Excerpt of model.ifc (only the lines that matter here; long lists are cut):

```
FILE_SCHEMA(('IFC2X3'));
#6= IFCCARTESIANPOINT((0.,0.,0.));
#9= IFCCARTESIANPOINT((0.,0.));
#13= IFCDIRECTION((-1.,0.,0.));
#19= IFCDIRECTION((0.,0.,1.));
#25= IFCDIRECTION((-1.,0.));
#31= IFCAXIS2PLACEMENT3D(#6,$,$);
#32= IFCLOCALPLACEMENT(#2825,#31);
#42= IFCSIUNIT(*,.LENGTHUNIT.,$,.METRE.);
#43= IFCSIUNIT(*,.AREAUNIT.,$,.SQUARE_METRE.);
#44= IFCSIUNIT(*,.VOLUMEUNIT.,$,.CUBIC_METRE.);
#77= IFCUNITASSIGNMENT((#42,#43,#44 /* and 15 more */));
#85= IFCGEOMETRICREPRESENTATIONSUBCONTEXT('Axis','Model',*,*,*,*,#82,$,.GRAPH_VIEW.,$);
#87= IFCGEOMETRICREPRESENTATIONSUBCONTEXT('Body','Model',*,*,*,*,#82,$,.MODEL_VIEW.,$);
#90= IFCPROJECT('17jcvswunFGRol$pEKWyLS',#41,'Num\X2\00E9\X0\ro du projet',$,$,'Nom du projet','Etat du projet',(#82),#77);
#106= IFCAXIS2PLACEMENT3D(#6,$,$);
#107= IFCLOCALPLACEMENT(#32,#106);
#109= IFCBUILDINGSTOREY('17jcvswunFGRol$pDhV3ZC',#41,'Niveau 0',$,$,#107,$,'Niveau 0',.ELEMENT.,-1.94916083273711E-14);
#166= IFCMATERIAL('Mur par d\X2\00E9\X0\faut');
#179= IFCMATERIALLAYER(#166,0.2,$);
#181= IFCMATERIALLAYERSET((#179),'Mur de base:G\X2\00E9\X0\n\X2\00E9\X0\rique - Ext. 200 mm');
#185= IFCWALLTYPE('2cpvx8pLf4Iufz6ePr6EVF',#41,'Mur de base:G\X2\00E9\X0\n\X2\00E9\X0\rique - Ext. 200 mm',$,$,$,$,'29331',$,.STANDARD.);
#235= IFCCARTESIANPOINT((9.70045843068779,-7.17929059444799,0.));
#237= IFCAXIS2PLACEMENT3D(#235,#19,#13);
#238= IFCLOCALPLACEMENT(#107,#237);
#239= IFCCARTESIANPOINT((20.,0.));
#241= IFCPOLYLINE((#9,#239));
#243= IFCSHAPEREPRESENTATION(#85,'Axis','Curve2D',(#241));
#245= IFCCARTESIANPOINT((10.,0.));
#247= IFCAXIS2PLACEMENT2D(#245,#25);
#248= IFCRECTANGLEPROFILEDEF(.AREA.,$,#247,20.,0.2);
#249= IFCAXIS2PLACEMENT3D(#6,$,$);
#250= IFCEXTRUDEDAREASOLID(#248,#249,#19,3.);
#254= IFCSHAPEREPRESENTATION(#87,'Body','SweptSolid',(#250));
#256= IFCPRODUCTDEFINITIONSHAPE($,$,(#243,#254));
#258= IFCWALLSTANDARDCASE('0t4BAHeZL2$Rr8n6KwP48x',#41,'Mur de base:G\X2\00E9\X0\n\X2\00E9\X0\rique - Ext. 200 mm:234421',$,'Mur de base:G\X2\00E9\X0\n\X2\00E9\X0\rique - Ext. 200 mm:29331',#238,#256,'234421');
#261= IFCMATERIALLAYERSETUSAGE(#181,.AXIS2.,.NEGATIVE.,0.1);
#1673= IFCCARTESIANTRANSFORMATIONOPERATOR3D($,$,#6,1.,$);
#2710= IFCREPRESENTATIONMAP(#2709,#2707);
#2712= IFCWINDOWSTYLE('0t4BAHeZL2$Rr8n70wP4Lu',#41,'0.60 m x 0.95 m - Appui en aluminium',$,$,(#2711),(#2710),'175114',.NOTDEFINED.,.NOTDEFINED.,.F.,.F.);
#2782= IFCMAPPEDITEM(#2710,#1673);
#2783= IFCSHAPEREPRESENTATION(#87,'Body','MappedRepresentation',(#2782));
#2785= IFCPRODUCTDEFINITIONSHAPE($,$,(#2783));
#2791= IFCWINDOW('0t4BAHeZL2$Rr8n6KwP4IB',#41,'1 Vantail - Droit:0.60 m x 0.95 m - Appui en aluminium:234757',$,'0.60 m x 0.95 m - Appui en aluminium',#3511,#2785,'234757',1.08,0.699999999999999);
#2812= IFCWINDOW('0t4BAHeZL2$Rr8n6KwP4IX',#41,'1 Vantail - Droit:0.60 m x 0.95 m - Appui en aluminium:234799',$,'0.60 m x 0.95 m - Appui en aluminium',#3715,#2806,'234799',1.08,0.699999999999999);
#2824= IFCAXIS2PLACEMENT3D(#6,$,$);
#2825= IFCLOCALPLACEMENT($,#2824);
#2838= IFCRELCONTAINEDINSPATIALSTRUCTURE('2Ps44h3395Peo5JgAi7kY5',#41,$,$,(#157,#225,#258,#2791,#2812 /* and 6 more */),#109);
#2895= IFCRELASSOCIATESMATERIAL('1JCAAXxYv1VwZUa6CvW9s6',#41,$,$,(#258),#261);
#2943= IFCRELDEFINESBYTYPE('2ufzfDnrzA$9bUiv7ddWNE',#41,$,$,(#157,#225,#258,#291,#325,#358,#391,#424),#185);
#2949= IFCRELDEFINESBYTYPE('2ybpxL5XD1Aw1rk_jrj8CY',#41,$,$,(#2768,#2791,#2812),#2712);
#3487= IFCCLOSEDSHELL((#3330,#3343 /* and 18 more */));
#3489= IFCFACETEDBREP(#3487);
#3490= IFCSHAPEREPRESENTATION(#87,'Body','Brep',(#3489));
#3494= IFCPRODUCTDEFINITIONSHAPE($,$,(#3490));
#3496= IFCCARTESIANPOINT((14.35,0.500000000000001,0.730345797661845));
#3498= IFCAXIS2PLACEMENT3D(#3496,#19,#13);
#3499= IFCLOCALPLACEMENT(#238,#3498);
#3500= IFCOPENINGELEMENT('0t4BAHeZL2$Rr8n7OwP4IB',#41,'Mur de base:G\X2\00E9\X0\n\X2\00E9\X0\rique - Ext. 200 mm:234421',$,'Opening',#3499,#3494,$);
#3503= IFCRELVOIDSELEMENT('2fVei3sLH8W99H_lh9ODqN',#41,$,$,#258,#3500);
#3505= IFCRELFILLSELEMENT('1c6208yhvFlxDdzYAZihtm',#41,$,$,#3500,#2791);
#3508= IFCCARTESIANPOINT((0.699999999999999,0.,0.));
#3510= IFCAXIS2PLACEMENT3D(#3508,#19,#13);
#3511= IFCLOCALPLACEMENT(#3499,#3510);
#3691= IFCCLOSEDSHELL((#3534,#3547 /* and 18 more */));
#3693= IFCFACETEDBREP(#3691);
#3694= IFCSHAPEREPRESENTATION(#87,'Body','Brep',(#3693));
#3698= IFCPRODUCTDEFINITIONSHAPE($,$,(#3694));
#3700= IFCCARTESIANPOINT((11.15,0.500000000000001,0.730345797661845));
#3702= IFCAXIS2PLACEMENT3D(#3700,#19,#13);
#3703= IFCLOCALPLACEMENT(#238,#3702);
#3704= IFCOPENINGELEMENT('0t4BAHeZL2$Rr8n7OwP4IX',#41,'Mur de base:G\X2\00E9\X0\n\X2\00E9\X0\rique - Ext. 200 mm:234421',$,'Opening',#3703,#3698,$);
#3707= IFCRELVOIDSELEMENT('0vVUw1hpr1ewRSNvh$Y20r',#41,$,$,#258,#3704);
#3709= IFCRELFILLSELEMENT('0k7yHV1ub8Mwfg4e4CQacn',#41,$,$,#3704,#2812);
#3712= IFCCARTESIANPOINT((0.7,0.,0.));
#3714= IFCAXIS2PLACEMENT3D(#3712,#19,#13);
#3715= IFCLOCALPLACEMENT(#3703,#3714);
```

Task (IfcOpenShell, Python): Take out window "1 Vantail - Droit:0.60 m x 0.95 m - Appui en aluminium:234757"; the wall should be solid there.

```python
import ifcopenshell
import ifcopenshell.api.feature
import ifcopenshell.api.root
import ifcopenshell.geom
import ifcopenshell.util.shape

model = ifcopenshell.open("model.ifc")
settings = ifcopenshell.geom.settings()


def volume(element):
    """Net volume in cubic metres, openings subtracted."""
    shape = ifcopenshell.geom.create_shape(settings, element)
    return ifcopenshell.util.shape.get_volume(shape.geometry)


window = model.by_id(2791)
opening = window.FillsVoids[0].RelatingOpeningElement
wall = opening.VoidsElements[0].RelatingBuildingElement
before = volume(wall)

ifcopenshell.api.root.remove_product(model, product=window)
ifcopenshell.api.feature.remove_feature(model, feature=opening)

after = volume(wall)

print(f"wall volume {before:.3f} -> {after:.3f} m3")

model.write("model-out.ifc")
```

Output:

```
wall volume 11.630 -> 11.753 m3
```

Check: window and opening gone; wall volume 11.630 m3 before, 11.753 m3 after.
